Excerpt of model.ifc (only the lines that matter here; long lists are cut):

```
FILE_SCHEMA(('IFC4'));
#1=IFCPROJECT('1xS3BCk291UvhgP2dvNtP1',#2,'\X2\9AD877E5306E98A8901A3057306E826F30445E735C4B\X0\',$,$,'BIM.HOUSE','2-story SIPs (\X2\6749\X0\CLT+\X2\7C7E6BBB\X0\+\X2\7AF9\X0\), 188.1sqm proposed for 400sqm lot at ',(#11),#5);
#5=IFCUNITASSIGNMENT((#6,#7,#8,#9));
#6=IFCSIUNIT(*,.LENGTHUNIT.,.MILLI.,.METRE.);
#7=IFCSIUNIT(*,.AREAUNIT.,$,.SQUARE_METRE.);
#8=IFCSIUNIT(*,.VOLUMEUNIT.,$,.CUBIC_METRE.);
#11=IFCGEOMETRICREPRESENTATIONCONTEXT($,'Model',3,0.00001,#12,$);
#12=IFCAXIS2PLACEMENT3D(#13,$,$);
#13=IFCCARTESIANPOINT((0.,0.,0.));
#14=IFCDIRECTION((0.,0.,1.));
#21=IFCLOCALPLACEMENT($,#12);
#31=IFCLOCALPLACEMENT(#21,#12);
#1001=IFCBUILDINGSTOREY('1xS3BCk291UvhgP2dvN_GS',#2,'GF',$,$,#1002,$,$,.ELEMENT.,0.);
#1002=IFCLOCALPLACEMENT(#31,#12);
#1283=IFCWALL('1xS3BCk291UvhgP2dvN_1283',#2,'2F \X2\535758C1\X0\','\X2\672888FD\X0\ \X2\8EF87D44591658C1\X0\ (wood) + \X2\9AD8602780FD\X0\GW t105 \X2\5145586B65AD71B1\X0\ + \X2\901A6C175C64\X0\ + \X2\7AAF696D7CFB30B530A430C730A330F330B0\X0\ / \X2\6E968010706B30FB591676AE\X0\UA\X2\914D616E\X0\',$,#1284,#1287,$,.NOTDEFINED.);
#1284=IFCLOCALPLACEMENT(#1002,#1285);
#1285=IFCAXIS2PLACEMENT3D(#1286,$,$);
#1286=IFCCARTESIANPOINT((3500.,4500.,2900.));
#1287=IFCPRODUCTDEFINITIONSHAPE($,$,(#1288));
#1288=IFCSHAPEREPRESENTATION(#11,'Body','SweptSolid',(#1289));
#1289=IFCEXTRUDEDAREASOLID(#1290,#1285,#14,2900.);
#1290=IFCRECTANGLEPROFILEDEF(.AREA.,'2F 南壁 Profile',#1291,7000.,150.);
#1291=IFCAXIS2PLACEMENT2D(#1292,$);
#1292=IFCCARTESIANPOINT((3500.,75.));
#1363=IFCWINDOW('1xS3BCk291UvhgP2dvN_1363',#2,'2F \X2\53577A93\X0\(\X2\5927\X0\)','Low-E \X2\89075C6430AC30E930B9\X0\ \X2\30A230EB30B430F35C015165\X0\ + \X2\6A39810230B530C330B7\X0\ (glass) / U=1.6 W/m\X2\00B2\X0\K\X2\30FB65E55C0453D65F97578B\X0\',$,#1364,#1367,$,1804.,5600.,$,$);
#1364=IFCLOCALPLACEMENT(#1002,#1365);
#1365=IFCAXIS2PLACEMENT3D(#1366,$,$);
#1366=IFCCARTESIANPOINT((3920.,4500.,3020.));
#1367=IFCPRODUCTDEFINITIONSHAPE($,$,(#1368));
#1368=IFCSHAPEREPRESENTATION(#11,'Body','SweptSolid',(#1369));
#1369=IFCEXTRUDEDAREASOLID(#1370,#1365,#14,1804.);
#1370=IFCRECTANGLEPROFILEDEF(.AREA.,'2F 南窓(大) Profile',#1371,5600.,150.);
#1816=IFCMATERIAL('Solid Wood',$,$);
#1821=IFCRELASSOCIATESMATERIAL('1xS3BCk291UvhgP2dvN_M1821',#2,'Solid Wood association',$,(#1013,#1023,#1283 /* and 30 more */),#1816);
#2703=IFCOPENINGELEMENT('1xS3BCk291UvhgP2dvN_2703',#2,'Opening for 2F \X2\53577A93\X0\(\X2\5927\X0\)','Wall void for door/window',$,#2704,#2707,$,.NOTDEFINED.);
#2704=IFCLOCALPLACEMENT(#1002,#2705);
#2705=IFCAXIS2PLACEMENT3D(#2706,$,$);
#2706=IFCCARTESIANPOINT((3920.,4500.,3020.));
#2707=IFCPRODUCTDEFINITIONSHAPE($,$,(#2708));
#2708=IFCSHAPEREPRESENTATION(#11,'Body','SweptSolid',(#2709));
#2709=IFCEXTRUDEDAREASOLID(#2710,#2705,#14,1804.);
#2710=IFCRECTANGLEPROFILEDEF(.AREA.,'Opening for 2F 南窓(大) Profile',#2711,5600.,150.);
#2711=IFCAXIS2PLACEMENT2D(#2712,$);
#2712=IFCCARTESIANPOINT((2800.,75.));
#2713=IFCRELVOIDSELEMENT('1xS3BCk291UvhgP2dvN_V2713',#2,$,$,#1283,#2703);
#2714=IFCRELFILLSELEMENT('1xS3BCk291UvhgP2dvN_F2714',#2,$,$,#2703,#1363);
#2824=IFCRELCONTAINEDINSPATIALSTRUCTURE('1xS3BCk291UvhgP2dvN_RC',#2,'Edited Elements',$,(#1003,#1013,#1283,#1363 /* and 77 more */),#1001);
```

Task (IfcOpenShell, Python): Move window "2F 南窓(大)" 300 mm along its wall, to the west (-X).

```python
import ifcopenshell
import ifcopenshell.api.geometry
import ifcopenshell.util.placement
import ifcopenshell.util.unit

model = ifcopenshell.open("model.ifc")
unit_scale = ifcopenshell.util.unit.calculate_unit_scale(model)

window = model.by_id(1363)
opening = window.FillsVoids[0].RelatingOpeningElement
wall = opening.VoidsElements[0].RelatingBuildingElement

wall_matrix = ifcopenshell.util.placement.get_local_placement(wall.ObjectPlacement)
shift = wall_matrix[:3, 0] * -0.3 / unit_scale
before = ifcopenshell.util.placement.get_local_placement(window.ObjectPlacement)[:3, 3].copy()

# The window is not placed relative to its opening, so move both.
for product in (opening, window):
    matrix = ifcopenshell.util.placement.get_local_placement(product.ObjectPlacement)
    matrix[:3, 3] += shift
    ifcopenshell.api.geometry.edit_object_placement(model, product=product, matrix=matrix, is_si=False)

after = ifcopenshell.util.placement.get_local_placement(window.ObjectPlacement)[:3, 3]
print("window moved by", (after - before).round(3) + 0.0)

model.write("model_updated.ifc")
```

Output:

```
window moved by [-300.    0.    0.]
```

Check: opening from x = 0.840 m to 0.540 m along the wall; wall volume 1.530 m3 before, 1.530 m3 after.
